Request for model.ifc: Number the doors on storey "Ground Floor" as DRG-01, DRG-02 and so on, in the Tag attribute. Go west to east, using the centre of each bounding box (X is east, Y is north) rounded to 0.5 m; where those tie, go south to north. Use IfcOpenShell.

First a look at what the model holds.

```python
import ifcopenshell
import ifcopenshell.util.element
import ifcopenshell.util.placement

model = ifcopenshell.open("model.ifc")
print(model.schema)
storey = next(s for s in model.by_type("IfcBuildingStorey") if s.Name == "Ground Floor")
doors = [e for e in ifcopenshell.util.element.get_decomposition(storey) if e.is_a("IfcDoor")]
for e in sorted(doors, key=lambda e: e.id()):
    origin = ifcopenshell.util.placement.get_local_placement(e.ObjectPlacement)[:3, 3]
    print(e.id(), e.Tag, e.Name, origin.round(2) + 0.0, sep=" | ")
```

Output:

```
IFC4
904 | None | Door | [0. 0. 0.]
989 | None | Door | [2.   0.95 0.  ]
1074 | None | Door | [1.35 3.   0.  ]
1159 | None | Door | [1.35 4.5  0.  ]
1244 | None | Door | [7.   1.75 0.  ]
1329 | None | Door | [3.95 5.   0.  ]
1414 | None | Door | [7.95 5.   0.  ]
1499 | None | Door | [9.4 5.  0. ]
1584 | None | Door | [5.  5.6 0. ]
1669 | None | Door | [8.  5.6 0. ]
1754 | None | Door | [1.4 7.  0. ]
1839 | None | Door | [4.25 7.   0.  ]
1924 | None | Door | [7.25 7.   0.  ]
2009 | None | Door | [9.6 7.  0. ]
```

```python
import ifcopenshell
import ifcopenshell.geom
import ifcopenshell.util.element
import ifcopenshell.util.shape

model = ifcopenshell.open("model.ifc")
settings = ifcopenshell.geom.settings()
settings.set("use-world-coords", True)


def centre(element):
    shape = ifcopenshell.geom.create_shape(settings, element)
    return ifcopenshell.util.shape.get_bbox_centroid(shape.geometry)


storey = next(s for s in model.by_type("IfcBuildingStorey") if s.Name == "Ground Floor")
doors = [e for e in ifcopenshell.util.element.get_decomposition(storey) if e.is_a("IfcDoor")]

# Insertion points can sit at a corner or the storey origin, so sort by the geometry (in metres).
centres = {e: centre(e) for e in doors}
doors.sort(key=lambda e: (round(centres[e][0] / 0.5), centres[e][1]))

for i, e in enumerate(doors, start=1):
    number = f"DRG-{i:02d}"
    e.Tag = number
    print(e.id(), number)

model.write("model_v2.ifc")
```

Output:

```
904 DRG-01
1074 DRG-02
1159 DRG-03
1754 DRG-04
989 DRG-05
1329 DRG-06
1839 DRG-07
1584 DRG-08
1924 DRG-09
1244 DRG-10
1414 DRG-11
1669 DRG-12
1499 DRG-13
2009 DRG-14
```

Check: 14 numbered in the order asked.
